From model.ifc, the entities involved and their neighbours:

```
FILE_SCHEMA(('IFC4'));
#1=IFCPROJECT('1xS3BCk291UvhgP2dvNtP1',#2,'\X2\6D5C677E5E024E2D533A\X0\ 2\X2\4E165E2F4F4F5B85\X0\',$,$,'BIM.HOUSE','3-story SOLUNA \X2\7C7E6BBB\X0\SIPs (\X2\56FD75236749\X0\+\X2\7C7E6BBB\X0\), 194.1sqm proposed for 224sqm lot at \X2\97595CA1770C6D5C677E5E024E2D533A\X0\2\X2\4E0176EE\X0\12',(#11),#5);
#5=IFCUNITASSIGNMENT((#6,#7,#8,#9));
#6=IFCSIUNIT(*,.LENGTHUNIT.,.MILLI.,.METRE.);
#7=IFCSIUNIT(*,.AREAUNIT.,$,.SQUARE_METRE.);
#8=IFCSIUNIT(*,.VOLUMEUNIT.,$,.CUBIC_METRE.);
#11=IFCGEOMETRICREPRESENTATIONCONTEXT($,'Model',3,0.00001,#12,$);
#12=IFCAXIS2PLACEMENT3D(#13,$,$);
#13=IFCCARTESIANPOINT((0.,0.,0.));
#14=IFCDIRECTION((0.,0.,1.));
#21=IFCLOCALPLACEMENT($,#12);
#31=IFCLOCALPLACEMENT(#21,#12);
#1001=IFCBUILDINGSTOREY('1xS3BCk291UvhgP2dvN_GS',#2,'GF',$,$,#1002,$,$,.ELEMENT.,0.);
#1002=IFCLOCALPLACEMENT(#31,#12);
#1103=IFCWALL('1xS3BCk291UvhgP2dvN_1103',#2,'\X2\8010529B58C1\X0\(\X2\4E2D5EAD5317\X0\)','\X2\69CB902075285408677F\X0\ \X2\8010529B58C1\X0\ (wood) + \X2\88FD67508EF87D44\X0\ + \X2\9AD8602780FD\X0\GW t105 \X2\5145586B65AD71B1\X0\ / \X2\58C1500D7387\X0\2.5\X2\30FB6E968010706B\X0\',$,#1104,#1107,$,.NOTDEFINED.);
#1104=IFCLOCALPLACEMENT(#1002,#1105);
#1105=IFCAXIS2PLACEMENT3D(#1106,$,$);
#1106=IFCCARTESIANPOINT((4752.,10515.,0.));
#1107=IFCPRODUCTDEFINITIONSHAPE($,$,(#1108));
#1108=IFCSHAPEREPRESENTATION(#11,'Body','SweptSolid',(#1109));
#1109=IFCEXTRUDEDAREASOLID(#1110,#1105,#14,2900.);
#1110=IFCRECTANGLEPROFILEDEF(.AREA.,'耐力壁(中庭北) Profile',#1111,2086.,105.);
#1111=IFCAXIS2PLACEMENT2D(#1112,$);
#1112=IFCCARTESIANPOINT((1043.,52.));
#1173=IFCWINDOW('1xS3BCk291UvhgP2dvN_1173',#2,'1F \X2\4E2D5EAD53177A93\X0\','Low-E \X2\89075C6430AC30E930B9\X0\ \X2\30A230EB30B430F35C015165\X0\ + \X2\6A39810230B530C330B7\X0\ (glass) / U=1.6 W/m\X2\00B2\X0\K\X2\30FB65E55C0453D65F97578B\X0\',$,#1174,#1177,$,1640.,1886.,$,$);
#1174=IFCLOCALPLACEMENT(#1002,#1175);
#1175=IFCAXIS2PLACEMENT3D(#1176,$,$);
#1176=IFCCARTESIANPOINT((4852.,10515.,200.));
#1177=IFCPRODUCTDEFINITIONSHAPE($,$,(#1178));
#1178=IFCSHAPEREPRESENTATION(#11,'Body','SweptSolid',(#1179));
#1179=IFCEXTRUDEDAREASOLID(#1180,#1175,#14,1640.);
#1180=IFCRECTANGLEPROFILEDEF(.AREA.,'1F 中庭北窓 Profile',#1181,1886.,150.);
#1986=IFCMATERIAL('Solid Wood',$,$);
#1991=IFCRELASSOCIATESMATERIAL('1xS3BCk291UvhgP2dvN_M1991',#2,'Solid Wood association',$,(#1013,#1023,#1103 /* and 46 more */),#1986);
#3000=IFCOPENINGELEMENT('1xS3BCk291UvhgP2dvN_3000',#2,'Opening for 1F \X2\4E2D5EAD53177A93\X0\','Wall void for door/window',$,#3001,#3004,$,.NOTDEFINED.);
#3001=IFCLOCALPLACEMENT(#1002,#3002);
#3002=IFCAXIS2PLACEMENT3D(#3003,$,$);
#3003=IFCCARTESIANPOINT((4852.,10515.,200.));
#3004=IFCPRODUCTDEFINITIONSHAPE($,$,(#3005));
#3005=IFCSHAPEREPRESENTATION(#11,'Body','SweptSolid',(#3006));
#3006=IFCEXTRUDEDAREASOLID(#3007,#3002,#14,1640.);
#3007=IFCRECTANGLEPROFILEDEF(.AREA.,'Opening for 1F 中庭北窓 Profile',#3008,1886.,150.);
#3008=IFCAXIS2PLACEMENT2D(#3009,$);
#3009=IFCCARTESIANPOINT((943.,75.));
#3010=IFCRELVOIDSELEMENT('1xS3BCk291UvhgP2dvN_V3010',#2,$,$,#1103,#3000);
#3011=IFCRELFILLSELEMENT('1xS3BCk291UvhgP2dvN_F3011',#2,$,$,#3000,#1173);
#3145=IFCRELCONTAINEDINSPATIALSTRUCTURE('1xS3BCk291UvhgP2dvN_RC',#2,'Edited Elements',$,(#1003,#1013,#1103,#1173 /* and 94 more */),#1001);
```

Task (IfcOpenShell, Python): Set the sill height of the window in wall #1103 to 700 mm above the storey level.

```python
import numpy as np
import ifcopenshell
import ifcopenshell.api.geometry
import ifcopenshell.geom
import ifcopenshell.util.element
import ifcopenshell.util.placement
import ifcopenshell.util.shape
import ifcopenshell.util.unit

model = ifcopenshell.open("model.ifc")
unit_scale = ifcopenshell.util.unit.calculate_unit_scale(model)

window = model.by_guid("1xS3BCk291UvhgP2dvN_1173")
opening = window.FillsVoids[0].RelatingOpeningElement
storey = ifcopenshell.util.element.get_container(window, ifc_class="IfcBuildingStorey")
level = ifcopenshell.util.placement.get_local_placement(storey.ObjectPlacement)[2, 3]

# The opening's origin need not be at the sill, so measure its lowest point.
shape = ifcopenshell.geom.create_shape(ifcopenshell.geom.settings(), opening)
bottom = ifcopenshell.util.shape.get_shape_bottom_elevation(shape, shape.geometry) / unit_scale
dz = level + 0.7 / unit_scale - bottom

shift = np.array([0.0, 0.0, dz])
# The window is not placed relative to its opening, so move both.
for product in (opening, window):
    matrix = ifcopenshell.util.placement.get_local_placement(product.ObjectPlacement)
    matrix[:3, 3] += shift
    ifcopenshell.api.geometry.edit_object_placement(model, product=product, matrix=matrix, is_si=False)

print(f"moved by {dz * unit_scale:+.3f} m")

model.write("model_rev.ifc")
```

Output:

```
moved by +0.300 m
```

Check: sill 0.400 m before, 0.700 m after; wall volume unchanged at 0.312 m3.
